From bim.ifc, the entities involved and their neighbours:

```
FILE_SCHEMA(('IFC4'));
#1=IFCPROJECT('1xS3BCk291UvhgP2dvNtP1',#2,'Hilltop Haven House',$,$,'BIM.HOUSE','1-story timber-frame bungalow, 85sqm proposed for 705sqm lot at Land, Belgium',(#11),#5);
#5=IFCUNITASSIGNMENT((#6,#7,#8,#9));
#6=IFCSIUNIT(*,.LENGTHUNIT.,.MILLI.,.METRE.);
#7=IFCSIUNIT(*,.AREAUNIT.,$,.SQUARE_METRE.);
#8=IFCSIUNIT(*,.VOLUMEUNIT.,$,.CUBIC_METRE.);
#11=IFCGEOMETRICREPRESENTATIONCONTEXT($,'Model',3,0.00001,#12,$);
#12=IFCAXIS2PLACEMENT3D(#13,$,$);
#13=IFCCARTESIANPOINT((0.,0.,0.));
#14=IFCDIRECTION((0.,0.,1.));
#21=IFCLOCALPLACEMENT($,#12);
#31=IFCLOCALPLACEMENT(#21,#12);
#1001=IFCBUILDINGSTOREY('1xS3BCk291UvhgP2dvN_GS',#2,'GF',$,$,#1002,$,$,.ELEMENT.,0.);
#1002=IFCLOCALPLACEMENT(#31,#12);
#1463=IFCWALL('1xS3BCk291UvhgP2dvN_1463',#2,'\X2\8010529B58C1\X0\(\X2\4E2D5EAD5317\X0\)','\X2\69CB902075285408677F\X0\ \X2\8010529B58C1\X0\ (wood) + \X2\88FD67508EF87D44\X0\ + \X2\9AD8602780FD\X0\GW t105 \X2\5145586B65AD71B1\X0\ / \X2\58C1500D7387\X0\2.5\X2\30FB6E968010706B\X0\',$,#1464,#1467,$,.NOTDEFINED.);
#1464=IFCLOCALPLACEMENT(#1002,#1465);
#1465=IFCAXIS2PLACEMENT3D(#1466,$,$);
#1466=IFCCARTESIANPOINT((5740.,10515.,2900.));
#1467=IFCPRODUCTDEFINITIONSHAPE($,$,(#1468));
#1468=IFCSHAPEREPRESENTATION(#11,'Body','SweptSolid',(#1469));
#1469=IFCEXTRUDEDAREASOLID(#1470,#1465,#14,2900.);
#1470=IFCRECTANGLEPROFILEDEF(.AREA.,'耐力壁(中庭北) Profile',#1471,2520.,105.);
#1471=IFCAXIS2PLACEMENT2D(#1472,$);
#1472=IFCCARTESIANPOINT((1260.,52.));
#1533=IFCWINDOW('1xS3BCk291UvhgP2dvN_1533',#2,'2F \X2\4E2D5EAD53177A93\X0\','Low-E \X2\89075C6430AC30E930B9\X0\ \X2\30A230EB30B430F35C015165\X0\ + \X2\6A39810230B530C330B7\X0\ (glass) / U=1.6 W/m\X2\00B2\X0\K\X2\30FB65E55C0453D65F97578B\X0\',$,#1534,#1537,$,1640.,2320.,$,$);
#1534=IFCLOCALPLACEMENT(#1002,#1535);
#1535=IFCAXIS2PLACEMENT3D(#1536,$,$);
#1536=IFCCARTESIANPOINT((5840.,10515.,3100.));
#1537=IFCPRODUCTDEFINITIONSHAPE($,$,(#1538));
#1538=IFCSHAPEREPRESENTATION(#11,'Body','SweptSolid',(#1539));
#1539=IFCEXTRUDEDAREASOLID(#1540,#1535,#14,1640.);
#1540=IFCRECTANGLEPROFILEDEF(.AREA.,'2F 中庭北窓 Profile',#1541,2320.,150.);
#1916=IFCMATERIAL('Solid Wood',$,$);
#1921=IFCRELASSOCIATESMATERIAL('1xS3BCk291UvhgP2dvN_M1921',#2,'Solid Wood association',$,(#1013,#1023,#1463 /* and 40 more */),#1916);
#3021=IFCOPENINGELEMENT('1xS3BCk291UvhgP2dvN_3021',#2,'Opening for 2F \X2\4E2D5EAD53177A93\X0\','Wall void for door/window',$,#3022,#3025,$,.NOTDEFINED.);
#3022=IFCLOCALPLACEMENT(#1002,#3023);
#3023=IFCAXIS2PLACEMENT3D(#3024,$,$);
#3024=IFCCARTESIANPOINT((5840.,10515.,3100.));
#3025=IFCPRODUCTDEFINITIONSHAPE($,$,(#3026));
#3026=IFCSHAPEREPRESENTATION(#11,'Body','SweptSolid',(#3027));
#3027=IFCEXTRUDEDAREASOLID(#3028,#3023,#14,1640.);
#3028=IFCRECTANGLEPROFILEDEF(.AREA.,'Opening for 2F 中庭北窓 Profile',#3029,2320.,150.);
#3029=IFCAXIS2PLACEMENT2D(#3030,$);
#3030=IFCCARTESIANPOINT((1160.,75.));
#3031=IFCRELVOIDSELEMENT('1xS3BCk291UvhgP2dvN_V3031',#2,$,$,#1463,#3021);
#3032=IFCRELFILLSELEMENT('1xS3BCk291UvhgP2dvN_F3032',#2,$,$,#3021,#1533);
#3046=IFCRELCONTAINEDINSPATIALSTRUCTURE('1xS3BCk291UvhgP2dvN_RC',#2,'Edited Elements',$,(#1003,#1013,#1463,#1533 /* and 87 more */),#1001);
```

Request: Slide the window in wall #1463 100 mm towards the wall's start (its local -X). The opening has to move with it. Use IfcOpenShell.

```python
import ifcopenshell
import ifcopenshell.api.geometry
import ifcopenshell.util.placement
import ifcopenshell.util.unit

model = ifcopenshell.open("bim.ifc")
unit_scale = ifcopenshell.util.unit.calculate_unit_scale(model)

window = model.by_guid("1xS3BCk291UvhgP2dvN_1533")
opening = window.FillsVoids[0].RelatingOpeningElement
wall = opening.VoidsElements[0].RelatingBuildingElement

wall_matrix = ifcopenshell.util.placement.get_local_placement(wall.ObjectPlacement)
shift = wall_matrix[:3, 0] * -0.1 / unit_scale
before = ifcopenshell.util.placement.get_local_placement(window.ObjectPlacement)[:3, 3].copy()

# The window is not placed relative to its opening, so move both.
for product in (opening, window):
    matrix = ifcopenshell.util.placement.get_local_placement(product.ObjectPlacement)
    matrix[:3, 3] += shift
    ifcopenshell.api.geometry.edit_object_placement(model, product=product, matrix=matrix, is_si=False)

after = ifcopenshell.util.placement.get_local_placement(window.ObjectPlacement)[:3, 3]
print("window moved by", (after - before).round(3) + 0.0)

model.write("bim-out.ifc")
```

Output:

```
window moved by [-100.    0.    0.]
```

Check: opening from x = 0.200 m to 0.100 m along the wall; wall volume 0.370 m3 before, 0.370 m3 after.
